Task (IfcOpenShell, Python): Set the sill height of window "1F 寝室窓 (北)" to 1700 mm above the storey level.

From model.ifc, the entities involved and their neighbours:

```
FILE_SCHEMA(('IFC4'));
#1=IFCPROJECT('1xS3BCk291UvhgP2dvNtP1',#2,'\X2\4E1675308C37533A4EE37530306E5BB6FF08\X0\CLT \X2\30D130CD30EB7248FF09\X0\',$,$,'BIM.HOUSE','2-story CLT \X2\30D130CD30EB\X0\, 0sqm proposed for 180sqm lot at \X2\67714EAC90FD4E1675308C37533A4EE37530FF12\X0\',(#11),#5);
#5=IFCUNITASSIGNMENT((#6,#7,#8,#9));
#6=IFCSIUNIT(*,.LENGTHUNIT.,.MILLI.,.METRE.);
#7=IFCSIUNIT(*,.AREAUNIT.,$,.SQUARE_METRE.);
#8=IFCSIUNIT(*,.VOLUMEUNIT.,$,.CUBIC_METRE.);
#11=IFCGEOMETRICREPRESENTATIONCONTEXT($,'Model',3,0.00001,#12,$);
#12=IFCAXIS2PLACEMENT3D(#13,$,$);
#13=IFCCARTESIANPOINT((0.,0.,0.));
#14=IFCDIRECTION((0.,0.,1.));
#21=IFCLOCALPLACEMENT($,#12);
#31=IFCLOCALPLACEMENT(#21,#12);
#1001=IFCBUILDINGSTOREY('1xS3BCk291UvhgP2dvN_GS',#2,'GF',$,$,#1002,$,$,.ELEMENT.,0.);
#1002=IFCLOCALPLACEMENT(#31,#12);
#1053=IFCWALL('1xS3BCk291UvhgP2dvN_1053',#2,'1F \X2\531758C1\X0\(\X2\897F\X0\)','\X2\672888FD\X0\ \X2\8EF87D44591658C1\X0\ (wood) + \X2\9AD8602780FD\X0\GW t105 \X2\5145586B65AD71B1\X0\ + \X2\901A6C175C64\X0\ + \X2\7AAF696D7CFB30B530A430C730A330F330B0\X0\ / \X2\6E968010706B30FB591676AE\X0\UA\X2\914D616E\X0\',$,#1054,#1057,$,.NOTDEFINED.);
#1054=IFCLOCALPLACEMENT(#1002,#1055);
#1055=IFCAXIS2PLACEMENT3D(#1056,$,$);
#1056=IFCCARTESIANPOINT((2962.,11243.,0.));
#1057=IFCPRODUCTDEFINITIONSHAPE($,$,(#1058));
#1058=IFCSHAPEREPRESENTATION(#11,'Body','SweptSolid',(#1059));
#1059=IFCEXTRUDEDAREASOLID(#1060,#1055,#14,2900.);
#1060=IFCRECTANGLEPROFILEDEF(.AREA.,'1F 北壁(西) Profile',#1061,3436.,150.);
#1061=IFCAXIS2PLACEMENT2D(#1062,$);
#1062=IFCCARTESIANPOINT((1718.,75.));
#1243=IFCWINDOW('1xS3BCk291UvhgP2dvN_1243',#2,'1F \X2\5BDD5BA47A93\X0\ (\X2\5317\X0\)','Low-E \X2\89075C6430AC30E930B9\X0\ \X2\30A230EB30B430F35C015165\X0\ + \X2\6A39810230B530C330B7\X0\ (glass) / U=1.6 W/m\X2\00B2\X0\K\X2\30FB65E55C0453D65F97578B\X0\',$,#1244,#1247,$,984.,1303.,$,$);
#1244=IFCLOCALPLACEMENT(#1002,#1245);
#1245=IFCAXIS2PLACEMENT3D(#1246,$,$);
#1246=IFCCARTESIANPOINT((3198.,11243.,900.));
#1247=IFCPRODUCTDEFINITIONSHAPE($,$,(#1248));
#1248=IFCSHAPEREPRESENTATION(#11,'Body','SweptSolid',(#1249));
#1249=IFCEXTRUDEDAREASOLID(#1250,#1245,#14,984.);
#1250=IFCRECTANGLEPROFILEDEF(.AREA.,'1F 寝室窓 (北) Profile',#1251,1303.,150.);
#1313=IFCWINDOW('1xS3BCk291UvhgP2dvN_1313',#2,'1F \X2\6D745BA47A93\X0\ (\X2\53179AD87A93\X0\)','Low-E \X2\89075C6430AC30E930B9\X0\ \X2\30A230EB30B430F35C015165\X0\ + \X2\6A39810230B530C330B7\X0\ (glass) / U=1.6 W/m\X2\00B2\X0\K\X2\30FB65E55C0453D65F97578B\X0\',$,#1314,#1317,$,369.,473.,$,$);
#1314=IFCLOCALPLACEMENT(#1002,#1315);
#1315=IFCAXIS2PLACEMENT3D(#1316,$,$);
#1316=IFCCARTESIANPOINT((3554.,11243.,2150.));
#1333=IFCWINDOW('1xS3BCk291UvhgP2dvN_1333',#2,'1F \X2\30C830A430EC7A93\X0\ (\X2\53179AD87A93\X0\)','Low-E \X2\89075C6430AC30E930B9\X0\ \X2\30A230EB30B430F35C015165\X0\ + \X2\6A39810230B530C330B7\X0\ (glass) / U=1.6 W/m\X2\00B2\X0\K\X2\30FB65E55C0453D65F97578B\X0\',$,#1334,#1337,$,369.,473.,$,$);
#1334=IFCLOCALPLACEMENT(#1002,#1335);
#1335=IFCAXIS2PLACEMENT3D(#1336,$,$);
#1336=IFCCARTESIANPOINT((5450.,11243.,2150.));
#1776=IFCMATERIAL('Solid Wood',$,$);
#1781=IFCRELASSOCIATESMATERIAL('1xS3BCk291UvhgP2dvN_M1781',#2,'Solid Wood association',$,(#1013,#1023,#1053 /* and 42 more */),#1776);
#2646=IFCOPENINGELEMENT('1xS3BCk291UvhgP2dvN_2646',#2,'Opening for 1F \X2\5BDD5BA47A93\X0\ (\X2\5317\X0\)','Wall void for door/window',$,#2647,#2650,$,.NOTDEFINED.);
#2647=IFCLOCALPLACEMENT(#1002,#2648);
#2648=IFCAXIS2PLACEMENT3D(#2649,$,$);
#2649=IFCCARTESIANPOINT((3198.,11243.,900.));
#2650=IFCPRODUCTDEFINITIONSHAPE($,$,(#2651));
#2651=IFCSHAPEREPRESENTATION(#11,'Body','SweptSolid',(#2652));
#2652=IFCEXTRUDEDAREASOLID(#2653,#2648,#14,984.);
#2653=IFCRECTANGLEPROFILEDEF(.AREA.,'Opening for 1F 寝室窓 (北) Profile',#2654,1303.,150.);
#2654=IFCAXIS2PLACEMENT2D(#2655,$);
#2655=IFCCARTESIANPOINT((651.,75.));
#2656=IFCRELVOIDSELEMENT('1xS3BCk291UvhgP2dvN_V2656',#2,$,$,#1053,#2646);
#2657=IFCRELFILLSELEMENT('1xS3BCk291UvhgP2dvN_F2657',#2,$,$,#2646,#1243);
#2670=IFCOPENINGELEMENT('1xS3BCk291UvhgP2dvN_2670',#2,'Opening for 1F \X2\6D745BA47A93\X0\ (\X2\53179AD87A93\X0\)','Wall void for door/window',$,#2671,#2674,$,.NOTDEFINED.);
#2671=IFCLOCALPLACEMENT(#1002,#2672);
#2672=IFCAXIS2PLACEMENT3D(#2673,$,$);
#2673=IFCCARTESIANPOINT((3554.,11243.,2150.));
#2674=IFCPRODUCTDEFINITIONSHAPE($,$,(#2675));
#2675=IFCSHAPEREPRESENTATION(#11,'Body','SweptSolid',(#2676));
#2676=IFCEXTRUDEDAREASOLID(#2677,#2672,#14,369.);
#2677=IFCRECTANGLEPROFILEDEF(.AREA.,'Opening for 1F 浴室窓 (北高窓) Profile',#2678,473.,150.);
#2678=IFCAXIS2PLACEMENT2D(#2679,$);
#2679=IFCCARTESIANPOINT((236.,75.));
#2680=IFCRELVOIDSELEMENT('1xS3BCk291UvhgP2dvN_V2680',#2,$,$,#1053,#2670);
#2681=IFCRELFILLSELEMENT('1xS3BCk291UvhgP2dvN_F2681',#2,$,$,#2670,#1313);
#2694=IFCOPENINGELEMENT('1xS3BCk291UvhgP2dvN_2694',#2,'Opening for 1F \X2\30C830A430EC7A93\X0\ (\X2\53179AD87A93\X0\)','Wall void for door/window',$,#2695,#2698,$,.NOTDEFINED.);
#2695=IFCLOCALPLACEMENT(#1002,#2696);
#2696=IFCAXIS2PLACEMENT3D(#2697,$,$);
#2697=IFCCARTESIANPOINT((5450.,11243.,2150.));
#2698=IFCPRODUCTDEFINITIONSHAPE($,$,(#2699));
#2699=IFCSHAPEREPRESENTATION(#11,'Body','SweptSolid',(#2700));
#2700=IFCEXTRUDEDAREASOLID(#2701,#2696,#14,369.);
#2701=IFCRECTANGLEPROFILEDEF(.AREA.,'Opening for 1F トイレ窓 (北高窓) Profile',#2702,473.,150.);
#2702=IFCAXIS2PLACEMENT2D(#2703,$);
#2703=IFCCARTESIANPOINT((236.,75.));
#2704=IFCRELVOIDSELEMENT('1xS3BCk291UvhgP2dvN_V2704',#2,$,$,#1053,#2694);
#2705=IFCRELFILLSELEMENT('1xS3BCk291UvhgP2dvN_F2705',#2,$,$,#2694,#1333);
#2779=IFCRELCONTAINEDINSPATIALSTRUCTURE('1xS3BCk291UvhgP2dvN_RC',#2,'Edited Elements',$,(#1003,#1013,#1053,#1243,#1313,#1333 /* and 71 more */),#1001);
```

```python
import numpy as np
import ifcopenshell
import ifcopenshell.api.geometry
import ifcopenshell.geom
import ifcopenshell.util.element
import ifcopenshell.util.placement
import ifcopenshell.util.shape
import ifcopenshell.util.unit

model = ifcopenshell.open("model.ifc")
unit_scale = ifcopenshell.util.unit.calculate_unit_scale(model)

window = model.by_id(1243)
opening = window.FillsVoids[0].RelatingOpeningElement
storey = ifcopenshell.util.element.get_container(window, ifc_class="IfcBuildingStorey")
level = ifcopenshell.util.placement.get_local_placement(storey.ObjectPlacement)[2, 3]

# The opening's origin need not be at the sill, so measure its lowest point.
shape = ifcopenshell.geom.create_shape(ifcopenshell.geom.settings(), opening)
bottom = ifcopenshell.util.shape.get_shape_bottom_elevation(shape, shape.geometry) / unit_scale
dz = level + 1.7 / unit_scale - bottom

shift = np.array([0.0, 0.0, dz])
# The window is not placed relative to its opening, so move both.
for product in (opening, window):
    matrix = ifcopenshell.util.placement.get_local_placement(product.ObjectPlacement)
    matrix[:3, 3] += shift
    ifcopenshell.api.geometry.edit_object_placement(model, product=product, matrix=matrix, is_si=False)

print(f"moved by {dz * unit_scale:+.3f} m")

model.write("model_updated.ifc")
```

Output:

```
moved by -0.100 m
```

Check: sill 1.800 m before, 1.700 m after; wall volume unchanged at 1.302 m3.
